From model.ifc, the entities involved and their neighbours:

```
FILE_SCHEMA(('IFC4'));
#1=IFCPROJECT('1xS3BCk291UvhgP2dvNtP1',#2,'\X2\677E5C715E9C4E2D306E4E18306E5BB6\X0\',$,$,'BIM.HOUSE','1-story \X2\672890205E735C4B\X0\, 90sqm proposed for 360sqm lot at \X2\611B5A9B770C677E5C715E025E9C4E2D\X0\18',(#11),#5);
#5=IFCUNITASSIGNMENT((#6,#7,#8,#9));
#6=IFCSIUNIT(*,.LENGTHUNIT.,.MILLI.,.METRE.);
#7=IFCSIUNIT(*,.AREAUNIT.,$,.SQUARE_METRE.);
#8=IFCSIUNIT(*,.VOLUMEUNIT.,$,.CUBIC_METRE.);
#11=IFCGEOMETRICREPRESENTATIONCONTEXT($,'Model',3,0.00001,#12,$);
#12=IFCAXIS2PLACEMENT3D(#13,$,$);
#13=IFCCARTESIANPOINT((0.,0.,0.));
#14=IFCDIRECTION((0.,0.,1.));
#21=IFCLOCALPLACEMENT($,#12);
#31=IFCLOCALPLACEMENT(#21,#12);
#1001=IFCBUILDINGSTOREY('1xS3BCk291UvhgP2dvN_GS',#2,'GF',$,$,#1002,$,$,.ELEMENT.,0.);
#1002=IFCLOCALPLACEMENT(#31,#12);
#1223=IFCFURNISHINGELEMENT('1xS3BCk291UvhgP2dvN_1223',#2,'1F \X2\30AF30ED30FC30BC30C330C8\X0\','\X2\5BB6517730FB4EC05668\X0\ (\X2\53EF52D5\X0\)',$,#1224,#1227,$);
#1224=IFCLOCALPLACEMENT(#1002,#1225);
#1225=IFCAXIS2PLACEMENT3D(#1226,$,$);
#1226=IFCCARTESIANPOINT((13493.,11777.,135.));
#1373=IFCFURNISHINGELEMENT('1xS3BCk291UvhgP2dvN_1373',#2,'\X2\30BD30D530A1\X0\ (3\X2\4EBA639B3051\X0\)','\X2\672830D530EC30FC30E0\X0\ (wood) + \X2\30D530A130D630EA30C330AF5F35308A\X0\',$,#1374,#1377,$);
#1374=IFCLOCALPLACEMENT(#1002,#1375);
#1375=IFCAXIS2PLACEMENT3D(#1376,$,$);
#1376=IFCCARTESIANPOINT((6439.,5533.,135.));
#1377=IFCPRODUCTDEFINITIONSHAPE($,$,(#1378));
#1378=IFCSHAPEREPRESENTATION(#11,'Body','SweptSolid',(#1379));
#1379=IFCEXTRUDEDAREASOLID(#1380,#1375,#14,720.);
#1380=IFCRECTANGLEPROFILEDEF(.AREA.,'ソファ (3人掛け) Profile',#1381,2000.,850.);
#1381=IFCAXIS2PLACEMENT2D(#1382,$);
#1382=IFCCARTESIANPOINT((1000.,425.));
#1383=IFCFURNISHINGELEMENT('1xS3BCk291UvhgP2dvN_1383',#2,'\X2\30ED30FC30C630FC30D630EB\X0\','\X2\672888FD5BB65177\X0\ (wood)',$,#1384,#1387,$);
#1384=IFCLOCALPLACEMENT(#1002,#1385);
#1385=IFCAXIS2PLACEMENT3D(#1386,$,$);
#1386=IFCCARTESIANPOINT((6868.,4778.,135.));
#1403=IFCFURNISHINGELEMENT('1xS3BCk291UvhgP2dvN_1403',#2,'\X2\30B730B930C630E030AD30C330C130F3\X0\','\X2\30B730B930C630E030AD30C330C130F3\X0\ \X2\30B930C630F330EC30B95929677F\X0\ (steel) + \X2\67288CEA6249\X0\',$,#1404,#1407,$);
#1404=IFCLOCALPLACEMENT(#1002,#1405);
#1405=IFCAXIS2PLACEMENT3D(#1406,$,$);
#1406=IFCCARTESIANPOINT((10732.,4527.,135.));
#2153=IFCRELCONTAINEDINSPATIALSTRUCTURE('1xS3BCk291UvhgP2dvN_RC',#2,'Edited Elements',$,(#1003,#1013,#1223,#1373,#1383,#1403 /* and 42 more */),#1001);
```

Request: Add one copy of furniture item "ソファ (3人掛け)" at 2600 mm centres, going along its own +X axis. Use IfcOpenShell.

```python
import ifcopenshell
import ifcopenshell.api.geometry
import ifcopenshell.api.root
import ifcopenshell.util.element
import ifcopenshell.util.placement

model = ifcopenshell.open("model.ifc")


def reuse_history(source, copy):
    """copy_class also copies each property set's owner history, people and application; keep the originals."""
    for rel in copy.IsDefinedBy:
        if rel.is_a("IfcRelDefinesByProperties") and (history := rel.RelatingPropertyDefinition.OwnerHistory):
            rel.RelatingPropertyDefinition.OwnerHistory = source.OwnerHistory
            ifcopenshell.util.element.remove_deep2(model, history)


source = model.by_id(1373)
base = ifcopenshell.util.placement.get_local_placement(source.ObjectPlacement)
step = base[:3, 0] * 2600.0

for i in range(1, 2):
    copy = ifcopenshell.api.root.copy_class(model, product=source)
    copy.Representation = ifcopenshell.util.element.copy_deep(
        model, source.Representation, exclude=["IfcGeometricRepresentationContext", "IfcRepresentationMap"]
    )
    reuse_history(source, copy)
    matrix = base.copy()
    matrix[:3, 3] += i * step
    print("added at", matrix[:3, 3].round(3) + 0.0)
    ifcopenshell.api.geometry.edit_object_placement(model, product=copy, matrix=matrix, is_si=False)

model.write("model_v2.ifc")
```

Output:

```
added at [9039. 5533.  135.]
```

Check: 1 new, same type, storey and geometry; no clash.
